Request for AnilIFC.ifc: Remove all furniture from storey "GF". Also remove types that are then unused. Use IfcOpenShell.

First a look at what the model holds.

```python
import ifcopenshell
import ifcopenshell.util.element

model = ifcopenshell.open("AnilIFC.ifc")
print(model.schema)
storey = next(s for s in model.by_type("IfcBuildingStorey") if s.Name == "GF")
furniture = [e for e in ifcopenshell.util.element.get_decomposition(storey) if e.is_a("IfcFurnishingElement")]
seen = {}
for e in furniture:
    element_type = ifcopenshell.util.element.get_type(e)
    name = element_type.Name if element_type not in (None, e) else None
    seen[name] = seen.get(name, 0) + 1
for name, count in sorted(seen.items(), key=str):
    print(count, "x", name)
```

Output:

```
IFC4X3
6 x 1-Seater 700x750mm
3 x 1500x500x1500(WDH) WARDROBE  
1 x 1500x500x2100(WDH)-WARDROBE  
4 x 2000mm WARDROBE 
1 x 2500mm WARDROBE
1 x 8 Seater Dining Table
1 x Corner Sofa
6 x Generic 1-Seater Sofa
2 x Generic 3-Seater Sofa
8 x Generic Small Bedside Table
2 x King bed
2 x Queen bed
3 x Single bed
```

```python
import ifcopenshell
import ifcopenshell.api.root
import ifcopenshell.util.element

model = ifcopenshell.open("AnilIFC.ifc")

storey = next(s for s in model.by_type("IfcBuildingStorey") if s.Name == "GF")
furniture = [e for e in ifcopenshell.util.element.get_decomposition(storey) if e.is_a("IfcFurnishingElement")]
types = {ifcopenshell.util.element.get_type(e) for e in furniture} - {None, *furniture}

for e in furniture:
    ifcopenshell.api.root.remove_product(model, product=e)
print(len(furniture), "removed")

unused = [t for t in types if not ifcopenshell.util.element.get_types(t)]
for t in unused:
    ifcopenshell.api.root.remove_product(model, product=t)
print(len(unused), "unused types removed")

model.write("AnilIFC_v2.ifc")
```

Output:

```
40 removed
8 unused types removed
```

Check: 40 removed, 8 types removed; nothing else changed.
